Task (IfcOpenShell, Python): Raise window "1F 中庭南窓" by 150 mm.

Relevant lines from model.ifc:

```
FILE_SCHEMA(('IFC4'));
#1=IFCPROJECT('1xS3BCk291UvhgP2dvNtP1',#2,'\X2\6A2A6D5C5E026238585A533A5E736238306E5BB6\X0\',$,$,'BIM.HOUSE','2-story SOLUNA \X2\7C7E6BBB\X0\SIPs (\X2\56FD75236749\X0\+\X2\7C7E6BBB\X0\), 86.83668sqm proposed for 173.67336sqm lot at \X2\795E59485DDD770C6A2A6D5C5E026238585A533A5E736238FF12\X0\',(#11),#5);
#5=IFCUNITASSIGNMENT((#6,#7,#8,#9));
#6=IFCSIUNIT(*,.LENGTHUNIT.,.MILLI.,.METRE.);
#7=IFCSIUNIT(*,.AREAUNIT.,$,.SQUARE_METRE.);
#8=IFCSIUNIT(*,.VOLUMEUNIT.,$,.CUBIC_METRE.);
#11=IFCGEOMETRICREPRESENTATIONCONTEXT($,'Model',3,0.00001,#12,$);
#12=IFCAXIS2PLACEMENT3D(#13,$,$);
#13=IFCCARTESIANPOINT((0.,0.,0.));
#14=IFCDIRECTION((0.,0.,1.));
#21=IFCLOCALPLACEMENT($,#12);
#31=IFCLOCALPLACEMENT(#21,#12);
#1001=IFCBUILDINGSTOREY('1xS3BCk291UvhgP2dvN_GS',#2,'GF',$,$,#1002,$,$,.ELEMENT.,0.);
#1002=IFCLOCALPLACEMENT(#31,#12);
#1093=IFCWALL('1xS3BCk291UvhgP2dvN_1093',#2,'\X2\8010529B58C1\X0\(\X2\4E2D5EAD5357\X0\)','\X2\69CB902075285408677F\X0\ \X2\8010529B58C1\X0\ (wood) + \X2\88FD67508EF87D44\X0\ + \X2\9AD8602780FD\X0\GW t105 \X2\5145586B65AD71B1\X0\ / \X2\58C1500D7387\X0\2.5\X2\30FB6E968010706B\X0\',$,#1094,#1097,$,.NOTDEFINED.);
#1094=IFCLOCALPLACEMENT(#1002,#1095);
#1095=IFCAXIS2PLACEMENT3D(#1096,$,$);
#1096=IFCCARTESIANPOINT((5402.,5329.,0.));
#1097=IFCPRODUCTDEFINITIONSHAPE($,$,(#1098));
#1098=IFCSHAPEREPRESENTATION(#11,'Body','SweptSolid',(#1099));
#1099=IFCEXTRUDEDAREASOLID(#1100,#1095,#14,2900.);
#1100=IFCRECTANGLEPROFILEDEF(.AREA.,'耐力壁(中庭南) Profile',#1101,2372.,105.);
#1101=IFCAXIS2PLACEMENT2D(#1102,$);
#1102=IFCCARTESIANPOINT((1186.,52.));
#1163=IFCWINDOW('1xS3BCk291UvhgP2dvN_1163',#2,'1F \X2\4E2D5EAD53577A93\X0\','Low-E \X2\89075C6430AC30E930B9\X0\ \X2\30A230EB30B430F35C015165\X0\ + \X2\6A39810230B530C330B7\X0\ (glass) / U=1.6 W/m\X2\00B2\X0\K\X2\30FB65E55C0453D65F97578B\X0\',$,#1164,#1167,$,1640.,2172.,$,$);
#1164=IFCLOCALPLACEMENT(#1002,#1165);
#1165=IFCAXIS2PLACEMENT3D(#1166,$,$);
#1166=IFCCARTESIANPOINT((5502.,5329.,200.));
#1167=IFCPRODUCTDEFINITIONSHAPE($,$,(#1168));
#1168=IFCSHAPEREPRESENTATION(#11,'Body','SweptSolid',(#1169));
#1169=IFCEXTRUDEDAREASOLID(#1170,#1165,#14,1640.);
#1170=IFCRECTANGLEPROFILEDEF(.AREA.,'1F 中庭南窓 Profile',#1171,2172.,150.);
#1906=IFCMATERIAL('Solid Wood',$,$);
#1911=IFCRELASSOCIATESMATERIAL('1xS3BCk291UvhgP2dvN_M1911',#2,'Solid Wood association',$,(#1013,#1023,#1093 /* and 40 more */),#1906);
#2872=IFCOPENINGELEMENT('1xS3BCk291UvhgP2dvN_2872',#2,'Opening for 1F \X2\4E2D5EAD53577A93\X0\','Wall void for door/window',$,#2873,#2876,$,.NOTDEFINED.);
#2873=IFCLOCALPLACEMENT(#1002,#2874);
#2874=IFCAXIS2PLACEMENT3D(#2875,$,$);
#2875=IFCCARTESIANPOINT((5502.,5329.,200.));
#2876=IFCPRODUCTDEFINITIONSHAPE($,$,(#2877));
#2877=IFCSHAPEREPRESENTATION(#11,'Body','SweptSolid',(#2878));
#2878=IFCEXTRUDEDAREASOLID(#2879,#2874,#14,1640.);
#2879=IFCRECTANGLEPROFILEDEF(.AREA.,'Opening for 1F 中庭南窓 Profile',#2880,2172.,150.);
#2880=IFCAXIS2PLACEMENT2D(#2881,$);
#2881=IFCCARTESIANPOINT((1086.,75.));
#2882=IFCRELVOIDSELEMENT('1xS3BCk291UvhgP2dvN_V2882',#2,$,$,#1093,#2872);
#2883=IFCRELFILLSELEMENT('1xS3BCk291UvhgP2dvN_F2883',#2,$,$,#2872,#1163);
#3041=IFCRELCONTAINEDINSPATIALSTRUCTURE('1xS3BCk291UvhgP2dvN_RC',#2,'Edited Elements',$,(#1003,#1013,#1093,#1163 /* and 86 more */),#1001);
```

```python
import numpy as np
import ifcopenshell
import ifcopenshell.api.geometry
import ifcopenshell.util.placement
import ifcopenshell.util.unit

model = ifcopenshell.open("model.ifc")
unit_scale = ifcopenshell.util.unit.calculate_unit_scale(model)

window = model.by_id(1163)
opening = window.FillsVoids[0].RelatingOpeningElement
dz = 150.0

shift = np.array([0.0, 0.0, dz])
# The window is not placed relative to its opening, so move both.
for product in (opening, window):
    matrix = ifcopenshell.util.placement.get_local_placement(product.ObjectPlacement)
    matrix[:3, 3] += shift
    ifcopenshell.api.geometry.edit_object_placement(model, product=product, matrix=matrix, is_si=False)

print(f"moved by {dz * unit_scale:+.3f} m")

model.write("model_edited.ifc")
```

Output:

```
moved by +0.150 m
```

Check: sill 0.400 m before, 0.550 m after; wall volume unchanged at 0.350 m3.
